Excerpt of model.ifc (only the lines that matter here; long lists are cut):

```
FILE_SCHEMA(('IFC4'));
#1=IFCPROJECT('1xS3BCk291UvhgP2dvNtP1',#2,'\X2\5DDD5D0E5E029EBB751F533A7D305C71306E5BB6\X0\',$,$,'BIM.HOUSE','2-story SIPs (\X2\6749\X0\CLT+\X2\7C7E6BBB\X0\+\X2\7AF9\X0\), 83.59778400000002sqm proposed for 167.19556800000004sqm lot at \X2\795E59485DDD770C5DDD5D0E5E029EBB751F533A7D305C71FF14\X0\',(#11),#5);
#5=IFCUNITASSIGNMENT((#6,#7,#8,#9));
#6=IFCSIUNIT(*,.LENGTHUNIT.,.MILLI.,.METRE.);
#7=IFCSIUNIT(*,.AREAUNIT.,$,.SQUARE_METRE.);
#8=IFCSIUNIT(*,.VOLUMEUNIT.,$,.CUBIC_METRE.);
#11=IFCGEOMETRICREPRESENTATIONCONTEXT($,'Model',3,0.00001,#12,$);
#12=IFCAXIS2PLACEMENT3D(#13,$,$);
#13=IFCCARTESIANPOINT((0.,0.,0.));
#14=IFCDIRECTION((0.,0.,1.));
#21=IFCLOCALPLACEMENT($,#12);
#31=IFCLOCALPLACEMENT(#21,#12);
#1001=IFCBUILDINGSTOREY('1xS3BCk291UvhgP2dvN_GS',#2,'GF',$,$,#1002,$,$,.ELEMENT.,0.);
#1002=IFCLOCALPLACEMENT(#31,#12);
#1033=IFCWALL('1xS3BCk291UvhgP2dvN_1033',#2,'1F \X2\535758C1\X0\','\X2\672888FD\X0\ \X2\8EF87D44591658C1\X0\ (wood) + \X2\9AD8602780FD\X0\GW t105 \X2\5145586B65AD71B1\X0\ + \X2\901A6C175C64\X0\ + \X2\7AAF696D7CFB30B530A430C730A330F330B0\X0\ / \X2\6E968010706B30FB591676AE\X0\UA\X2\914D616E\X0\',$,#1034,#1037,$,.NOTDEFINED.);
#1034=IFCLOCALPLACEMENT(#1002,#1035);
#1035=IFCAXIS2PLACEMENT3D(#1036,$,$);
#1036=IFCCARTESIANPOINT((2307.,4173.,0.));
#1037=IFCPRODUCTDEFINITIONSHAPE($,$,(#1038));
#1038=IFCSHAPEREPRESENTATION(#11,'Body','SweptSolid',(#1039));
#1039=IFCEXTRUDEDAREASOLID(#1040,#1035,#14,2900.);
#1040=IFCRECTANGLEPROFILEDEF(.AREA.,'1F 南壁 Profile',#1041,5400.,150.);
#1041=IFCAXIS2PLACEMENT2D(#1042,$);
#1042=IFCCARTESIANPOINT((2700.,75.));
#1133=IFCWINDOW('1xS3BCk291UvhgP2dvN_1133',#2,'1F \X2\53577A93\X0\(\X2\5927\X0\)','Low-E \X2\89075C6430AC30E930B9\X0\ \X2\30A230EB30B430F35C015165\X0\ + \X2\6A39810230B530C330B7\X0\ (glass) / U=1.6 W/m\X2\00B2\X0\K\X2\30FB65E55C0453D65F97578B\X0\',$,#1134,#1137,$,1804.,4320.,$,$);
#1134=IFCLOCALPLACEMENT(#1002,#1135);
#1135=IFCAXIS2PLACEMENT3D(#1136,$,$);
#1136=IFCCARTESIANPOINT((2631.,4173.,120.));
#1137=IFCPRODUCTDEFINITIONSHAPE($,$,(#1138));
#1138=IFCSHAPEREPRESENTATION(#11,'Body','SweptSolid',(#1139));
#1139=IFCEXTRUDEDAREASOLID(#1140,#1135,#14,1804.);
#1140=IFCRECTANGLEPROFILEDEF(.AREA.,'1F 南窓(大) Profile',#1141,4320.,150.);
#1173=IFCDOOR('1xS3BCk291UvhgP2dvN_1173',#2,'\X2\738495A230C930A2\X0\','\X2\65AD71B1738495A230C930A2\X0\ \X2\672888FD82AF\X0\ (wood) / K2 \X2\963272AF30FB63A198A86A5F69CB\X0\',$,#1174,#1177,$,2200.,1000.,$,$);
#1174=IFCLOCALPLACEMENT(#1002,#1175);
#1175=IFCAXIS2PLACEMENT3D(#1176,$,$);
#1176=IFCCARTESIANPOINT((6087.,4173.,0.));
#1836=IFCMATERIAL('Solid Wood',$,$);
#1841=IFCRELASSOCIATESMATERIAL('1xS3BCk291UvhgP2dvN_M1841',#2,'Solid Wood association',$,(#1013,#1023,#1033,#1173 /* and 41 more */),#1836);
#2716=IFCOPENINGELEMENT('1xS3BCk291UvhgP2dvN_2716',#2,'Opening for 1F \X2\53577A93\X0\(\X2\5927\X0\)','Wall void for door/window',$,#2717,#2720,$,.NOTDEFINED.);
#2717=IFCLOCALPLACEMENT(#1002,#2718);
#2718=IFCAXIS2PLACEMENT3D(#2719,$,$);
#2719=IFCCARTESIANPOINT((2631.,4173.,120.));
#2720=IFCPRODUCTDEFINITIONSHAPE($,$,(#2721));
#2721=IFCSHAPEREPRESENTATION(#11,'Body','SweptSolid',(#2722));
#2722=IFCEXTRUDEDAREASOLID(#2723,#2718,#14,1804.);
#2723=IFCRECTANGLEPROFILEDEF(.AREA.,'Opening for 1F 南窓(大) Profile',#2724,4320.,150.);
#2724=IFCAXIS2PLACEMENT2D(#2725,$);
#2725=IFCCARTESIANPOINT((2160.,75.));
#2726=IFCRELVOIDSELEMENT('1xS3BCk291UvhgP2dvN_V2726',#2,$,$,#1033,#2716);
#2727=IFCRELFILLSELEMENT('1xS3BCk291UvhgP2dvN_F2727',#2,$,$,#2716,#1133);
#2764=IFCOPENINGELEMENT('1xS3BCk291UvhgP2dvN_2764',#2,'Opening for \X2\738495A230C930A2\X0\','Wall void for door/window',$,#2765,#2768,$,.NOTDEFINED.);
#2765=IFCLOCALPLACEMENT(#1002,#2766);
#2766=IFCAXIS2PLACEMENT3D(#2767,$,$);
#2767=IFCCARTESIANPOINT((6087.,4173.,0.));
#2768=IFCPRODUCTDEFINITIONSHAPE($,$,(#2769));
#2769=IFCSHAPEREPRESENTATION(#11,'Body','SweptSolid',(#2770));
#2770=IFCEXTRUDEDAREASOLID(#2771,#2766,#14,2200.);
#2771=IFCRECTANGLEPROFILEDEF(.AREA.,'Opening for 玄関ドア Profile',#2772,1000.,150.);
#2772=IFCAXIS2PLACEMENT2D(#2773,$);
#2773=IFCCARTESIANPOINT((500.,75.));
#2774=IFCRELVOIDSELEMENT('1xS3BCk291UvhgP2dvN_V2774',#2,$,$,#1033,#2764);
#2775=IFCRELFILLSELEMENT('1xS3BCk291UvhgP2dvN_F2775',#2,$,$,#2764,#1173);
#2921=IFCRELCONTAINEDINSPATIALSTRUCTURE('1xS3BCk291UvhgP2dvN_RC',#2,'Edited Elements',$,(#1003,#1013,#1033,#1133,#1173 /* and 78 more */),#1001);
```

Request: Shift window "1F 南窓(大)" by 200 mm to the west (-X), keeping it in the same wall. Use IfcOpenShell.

```python
import ifcopenshell
import ifcopenshell.api.geometry
import ifcopenshell.util.placement
import ifcopenshell.util.unit

model = ifcopenshell.open("model.ifc")
unit_scale = ifcopenshell.util.unit.calculate_unit_scale(model)

window = model.by_guid("1xS3BCk291UvhgP2dvN_1133")
opening = window.FillsVoids[0].RelatingOpeningElement
wall = opening.VoidsElements[0].RelatingBuildingElement

wall_matrix = ifcopenshell.util.placement.get_local_placement(wall.ObjectPlacement)
shift = wall_matrix[:3, 0] * -0.2 / unit_scale
before = ifcopenshell.util.placement.get_local_placement(window.ObjectPlacement)[:3, 3].copy()

# The window is not placed relative to its opening, so move both.
for product in (opening, window):
    matrix = ifcopenshell.util.placement.get_local_placement(product.ObjectPlacement)
    matrix[:3, 3] += shift
    ifcopenshell.api.geometry.edit_object_placement(model, product=product, matrix=matrix, is_si=False)

after = ifcopenshell.util.placement.get_local_placement(window.ObjectPlacement)[:3, 3]
print("window moved by", (after - before).round(3) + 0.0)

model.write("model_v2.ifc")
```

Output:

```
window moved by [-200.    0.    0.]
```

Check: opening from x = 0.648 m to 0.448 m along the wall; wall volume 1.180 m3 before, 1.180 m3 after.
